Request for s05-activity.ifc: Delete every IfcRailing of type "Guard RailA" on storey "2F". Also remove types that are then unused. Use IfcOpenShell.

First a look at what the model holds.

```python
import ifcopenshell
import ifcopenshell.util.element

model = ifcopenshell.open("s05-activity.ifc")
print(model.schema)
storey = next(s for s in model.by_type("IfcBuildingStorey") if s.Name == "2F")
railings = [e for e in ifcopenshell.util.element.get_decomposition(storey) if e.is_a("IfcRailing")]
seen = {}
for e in railings:
    element_type = ifcopenshell.util.element.get_type(e)
    name = element_type.Name if element_type not in (None, e) else None
    seen[name] = seen.get(name, 0) + 1
for name, count in sorted(seen.items(), key=str):
    print(count, "x", name)
```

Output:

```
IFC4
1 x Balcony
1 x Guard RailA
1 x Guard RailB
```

```python
import ifcopenshell
import ifcopenshell.api.root
import ifcopenshell.util.element

model = ifcopenshell.open("s05-activity.ifc")

storey = next(s for s in model.by_type("IfcBuildingStorey") if s.Name == "2F")
railings = [e for e in ifcopenshell.util.element.get_decomposition(storey) if e.is_a("IfcRailing")]
targets = [e for e in railings if (t := ifcopenshell.util.element.get_type(e)) not in (None, e) and t.Name == "Guard RailA"]
types = {ifcopenshell.util.element.get_type(e) for e in targets} - {None, *targets}

for e in targets:
    ifcopenshell.api.root.remove_product(model, product=e)
print(len(targets), "removed")

unused = [t for t in types if not ifcopenshell.util.element.get_types(t)]
for t in unused:
    ifcopenshell.api.root.remove_product(model, product=t)
print(len(unused), "unused types removed")

model.write("s05-activity_v2.ifc")
```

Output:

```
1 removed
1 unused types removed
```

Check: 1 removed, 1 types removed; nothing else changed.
